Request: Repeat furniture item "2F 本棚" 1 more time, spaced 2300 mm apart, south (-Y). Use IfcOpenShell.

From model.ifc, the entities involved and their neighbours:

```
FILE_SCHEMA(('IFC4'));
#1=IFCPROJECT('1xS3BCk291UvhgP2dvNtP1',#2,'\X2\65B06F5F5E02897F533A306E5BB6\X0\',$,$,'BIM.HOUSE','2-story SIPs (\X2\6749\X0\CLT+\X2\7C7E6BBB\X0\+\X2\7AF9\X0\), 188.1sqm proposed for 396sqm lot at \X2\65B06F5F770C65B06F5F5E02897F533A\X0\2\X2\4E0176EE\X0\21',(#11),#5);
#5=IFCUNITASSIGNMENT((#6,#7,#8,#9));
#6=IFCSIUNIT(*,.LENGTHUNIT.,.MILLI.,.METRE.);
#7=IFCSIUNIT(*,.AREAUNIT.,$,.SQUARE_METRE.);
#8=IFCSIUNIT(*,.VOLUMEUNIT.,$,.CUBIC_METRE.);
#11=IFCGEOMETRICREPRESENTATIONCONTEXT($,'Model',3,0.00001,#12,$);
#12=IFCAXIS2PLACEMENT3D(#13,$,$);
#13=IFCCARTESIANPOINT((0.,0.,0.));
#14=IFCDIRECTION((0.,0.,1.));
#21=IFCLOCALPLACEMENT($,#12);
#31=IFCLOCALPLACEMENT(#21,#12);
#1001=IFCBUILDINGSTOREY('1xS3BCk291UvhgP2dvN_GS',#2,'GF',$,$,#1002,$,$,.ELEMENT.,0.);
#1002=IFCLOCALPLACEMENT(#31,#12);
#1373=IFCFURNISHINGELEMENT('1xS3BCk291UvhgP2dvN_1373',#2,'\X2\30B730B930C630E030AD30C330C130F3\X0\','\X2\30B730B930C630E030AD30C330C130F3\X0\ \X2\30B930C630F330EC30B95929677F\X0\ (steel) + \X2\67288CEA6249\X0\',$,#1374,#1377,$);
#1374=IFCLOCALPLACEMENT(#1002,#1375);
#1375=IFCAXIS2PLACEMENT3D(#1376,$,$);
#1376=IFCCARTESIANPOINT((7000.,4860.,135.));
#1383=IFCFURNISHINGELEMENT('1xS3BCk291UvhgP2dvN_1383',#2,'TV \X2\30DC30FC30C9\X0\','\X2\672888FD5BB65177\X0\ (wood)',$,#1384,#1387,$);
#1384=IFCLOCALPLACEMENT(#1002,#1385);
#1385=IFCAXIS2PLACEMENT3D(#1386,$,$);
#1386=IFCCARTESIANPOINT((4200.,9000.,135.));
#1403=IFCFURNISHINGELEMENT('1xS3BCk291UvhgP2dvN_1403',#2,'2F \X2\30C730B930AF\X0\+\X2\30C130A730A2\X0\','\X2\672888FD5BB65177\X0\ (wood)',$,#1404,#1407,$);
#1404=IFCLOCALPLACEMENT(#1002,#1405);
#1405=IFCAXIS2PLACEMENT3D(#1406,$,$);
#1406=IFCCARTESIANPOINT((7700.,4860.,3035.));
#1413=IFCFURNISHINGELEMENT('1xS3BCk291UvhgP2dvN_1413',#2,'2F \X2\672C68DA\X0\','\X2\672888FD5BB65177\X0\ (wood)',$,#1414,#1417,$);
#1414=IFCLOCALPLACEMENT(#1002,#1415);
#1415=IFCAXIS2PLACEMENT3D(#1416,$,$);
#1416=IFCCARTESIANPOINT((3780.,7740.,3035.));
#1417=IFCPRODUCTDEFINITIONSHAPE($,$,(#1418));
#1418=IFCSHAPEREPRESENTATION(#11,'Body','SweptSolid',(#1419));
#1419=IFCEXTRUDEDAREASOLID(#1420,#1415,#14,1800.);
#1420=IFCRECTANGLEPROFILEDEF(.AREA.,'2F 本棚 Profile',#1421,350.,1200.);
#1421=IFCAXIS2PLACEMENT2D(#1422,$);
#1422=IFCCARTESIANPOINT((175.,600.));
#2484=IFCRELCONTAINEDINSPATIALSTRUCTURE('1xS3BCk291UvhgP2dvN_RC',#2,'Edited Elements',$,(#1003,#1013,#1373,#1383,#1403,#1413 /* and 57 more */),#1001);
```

```python
import numpy as np
import ifcopenshell
import ifcopenshell.api.geometry
import ifcopenshell.api.root
import ifcopenshell.util.element
import ifcopenshell.util.placement

model = ifcopenshell.open("model.ifc")


def reuse_history(source, copy):
    """copy_class also copies each property set's owner history, people and application; keep the originals."""
    for rel in copy.IsDefinedBy:
        if rel.is_a("IfcRelDefinesByProperties") and (history := rel.RelatingPropertyDefinition.OwnerHistory):
            rel.RelatingPropertyDefinition.OwnerHistory = source.OwnerHistory
            ifcopenshell.util.element.remove_deep2(model, history)


source = model.by_guid("1xS3BCk291UvhgP2dvN_1413")
base = ifcopenshell.util.placement.get_local_placement(source.ObjectPlacement)
step = np.array([0.0, -1.0, 0.0]) * 2300.0

for i in range(1, 2):
    copy = ifcopenshell.api.root.copy_class(model, product=source)
    copy.Representation = ifcopenshell.util.element.copy_deep(
        model, source.Representation, exclude=["IfcGeometricRepresentationContext", "IfcRepresentationMap"]
    )
    reuse_history(source, copy)
    matrix = base.copy()
    matrix[:3, 3] += i * step
    print("added at", matrix[:3, 3].round(3) + 0.0)
    ifcopenshell.api.geometry.edit_object_placement(model, product=copy, matrix=matrix, is_si=False)

model.write("model_rev.ifc")
```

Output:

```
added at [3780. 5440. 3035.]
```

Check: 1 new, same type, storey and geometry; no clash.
